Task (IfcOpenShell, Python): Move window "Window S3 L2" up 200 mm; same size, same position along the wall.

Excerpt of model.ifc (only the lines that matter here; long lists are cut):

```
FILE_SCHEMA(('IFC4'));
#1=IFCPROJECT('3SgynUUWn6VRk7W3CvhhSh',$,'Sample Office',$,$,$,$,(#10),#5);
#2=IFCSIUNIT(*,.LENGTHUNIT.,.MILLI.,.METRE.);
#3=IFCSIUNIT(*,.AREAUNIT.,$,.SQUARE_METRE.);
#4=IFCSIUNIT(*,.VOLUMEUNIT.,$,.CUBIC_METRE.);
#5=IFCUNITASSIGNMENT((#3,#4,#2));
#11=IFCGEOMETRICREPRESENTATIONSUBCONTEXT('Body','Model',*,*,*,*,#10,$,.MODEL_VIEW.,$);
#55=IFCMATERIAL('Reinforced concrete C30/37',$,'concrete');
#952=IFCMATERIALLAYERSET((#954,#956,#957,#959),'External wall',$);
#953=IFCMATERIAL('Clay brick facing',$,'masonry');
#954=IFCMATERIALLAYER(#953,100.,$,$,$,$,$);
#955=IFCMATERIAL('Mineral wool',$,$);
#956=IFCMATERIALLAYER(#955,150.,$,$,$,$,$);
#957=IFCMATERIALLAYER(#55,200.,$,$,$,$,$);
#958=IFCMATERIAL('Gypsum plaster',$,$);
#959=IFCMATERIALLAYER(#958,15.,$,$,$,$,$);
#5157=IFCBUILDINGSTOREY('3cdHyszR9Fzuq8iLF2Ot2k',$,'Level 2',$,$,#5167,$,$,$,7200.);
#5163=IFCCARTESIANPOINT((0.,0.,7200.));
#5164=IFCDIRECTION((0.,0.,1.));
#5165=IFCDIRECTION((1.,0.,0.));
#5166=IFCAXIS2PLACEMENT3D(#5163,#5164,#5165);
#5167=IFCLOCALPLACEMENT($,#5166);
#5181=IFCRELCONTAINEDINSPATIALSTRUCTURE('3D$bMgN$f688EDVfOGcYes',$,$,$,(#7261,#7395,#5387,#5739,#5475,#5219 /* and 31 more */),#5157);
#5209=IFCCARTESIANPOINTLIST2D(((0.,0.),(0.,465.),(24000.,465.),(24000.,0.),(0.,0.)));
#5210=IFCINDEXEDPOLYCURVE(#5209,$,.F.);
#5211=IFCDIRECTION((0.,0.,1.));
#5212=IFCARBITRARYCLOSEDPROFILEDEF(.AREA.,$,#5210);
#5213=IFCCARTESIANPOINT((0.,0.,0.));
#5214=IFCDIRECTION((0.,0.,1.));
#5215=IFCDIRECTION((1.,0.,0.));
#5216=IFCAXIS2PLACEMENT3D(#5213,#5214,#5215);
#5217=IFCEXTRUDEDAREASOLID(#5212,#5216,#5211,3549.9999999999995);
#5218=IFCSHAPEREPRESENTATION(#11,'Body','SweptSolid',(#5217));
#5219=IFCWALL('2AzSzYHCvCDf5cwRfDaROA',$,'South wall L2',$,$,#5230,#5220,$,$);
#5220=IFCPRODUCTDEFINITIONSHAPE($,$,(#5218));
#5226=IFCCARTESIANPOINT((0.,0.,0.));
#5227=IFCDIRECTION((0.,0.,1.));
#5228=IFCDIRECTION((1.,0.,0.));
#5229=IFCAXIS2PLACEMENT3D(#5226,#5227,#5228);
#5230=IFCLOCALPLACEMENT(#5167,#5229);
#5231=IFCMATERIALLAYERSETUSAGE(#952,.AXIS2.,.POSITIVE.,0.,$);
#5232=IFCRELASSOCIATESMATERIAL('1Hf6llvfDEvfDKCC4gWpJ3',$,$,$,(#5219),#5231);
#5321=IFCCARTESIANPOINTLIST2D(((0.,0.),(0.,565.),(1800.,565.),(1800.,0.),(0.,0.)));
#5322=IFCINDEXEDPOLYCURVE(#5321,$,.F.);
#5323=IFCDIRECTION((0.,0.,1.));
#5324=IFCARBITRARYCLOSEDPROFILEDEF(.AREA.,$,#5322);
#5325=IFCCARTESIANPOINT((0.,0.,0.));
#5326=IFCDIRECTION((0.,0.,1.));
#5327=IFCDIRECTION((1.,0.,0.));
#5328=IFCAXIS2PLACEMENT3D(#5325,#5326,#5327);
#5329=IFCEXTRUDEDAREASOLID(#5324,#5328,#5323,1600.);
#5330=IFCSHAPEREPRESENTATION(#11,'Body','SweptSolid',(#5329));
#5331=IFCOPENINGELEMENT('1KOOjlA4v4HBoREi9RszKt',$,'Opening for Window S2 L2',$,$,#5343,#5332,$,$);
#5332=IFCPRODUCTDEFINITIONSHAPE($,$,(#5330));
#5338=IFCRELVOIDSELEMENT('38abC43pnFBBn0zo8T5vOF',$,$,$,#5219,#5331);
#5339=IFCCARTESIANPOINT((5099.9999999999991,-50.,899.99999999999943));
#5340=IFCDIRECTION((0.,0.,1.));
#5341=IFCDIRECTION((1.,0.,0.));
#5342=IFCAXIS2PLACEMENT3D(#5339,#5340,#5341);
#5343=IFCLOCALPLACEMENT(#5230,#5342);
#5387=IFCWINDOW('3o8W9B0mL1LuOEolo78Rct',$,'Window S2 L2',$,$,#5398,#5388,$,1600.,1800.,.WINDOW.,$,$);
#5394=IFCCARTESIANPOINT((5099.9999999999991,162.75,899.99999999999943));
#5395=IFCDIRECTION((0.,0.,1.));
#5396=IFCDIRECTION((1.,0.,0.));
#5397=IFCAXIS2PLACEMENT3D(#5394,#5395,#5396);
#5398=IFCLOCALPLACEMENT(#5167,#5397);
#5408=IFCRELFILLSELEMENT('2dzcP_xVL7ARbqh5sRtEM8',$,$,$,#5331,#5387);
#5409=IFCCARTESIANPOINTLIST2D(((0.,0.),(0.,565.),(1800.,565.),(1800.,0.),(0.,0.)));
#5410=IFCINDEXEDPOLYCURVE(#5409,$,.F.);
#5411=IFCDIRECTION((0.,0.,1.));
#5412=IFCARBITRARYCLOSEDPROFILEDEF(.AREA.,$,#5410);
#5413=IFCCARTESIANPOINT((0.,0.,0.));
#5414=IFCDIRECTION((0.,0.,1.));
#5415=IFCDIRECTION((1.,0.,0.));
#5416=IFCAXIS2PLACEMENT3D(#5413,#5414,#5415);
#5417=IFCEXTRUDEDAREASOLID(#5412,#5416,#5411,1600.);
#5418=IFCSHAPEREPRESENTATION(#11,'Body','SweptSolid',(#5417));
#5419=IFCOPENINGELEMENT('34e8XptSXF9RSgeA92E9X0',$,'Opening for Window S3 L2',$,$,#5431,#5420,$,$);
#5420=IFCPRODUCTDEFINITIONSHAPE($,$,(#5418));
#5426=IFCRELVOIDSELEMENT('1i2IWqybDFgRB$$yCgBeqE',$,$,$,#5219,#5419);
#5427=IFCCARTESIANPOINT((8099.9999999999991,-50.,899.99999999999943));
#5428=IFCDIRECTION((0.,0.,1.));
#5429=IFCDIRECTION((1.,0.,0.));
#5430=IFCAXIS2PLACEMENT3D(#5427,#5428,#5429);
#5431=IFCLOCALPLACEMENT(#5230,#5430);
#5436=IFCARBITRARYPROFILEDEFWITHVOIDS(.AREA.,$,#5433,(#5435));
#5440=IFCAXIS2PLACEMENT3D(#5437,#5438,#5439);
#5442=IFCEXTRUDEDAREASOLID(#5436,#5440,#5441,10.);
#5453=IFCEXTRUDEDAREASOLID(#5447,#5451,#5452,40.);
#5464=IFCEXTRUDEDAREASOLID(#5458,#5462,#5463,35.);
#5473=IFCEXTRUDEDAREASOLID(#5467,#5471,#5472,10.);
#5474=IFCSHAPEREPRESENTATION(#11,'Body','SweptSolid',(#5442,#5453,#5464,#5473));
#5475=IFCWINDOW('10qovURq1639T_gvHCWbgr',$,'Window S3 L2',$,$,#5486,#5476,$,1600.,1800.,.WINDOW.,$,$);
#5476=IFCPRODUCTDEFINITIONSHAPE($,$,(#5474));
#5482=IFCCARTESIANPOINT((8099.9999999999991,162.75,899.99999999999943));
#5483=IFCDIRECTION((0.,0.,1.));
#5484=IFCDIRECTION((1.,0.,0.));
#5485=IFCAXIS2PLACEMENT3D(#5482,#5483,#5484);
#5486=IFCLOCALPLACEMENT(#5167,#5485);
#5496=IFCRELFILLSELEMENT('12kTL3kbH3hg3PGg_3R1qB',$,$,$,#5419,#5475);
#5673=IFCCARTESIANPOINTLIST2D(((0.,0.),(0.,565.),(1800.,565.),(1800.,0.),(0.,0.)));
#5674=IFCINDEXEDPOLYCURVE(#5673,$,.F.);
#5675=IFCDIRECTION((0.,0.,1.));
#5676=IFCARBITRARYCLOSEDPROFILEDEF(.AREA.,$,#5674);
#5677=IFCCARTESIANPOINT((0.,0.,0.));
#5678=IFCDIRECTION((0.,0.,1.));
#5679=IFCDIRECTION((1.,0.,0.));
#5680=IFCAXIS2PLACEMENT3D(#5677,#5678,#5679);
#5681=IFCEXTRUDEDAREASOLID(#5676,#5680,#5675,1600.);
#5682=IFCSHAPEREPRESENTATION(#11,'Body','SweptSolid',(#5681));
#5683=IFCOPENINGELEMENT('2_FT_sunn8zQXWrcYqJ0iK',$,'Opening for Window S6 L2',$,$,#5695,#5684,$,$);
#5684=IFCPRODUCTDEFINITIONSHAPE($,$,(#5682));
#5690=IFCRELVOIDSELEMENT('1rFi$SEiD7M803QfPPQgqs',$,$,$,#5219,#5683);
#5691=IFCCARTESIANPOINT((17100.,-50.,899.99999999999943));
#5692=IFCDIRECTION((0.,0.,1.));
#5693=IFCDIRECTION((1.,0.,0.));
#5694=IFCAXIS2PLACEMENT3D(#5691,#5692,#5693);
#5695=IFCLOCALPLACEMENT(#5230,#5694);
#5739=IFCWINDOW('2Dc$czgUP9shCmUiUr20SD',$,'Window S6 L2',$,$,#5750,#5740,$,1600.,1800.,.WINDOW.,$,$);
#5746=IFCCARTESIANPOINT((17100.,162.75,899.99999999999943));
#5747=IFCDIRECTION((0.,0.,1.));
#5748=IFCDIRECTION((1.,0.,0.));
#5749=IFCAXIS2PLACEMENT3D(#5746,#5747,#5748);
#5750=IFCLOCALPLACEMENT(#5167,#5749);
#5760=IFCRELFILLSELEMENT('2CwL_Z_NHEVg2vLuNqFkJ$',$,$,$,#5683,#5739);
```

```python
import numpy as np
import ifcopenshell
import ifcopenshell.api.geometry
import ifcopenshell.util.placement
import ifcopenshell.util.unit

model = ifcopenshell.open("model.ifc")
unit_scale = ifcopenshell.util.unit.calculate_unit_scale(model)

window = model.by_guid("10qovURq1639T_gvHCWbgr")
opening = window.FillsVoids[0].RelatingOpeningElement
dz = 0.2 / unit_scale

shift = np.array([0.0, 0.0, dz])
# The window is not placed relative to its opening, so move both.
for product in (opening, window):
    matrix = ifcopenshell.util.placement.get_local_placement(product.ObjectPlacement)
    matrix[:3, 3] += shift
    ifcopenshell.api.geometry.edit_object_placement(model, product=product, matrix=matrix, is_si=False)

print(f"moved by {dz * unit_scale:+.3f} m")

model.write("model_edited.ifc")
```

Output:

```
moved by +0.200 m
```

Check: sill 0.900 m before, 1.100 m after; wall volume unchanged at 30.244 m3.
